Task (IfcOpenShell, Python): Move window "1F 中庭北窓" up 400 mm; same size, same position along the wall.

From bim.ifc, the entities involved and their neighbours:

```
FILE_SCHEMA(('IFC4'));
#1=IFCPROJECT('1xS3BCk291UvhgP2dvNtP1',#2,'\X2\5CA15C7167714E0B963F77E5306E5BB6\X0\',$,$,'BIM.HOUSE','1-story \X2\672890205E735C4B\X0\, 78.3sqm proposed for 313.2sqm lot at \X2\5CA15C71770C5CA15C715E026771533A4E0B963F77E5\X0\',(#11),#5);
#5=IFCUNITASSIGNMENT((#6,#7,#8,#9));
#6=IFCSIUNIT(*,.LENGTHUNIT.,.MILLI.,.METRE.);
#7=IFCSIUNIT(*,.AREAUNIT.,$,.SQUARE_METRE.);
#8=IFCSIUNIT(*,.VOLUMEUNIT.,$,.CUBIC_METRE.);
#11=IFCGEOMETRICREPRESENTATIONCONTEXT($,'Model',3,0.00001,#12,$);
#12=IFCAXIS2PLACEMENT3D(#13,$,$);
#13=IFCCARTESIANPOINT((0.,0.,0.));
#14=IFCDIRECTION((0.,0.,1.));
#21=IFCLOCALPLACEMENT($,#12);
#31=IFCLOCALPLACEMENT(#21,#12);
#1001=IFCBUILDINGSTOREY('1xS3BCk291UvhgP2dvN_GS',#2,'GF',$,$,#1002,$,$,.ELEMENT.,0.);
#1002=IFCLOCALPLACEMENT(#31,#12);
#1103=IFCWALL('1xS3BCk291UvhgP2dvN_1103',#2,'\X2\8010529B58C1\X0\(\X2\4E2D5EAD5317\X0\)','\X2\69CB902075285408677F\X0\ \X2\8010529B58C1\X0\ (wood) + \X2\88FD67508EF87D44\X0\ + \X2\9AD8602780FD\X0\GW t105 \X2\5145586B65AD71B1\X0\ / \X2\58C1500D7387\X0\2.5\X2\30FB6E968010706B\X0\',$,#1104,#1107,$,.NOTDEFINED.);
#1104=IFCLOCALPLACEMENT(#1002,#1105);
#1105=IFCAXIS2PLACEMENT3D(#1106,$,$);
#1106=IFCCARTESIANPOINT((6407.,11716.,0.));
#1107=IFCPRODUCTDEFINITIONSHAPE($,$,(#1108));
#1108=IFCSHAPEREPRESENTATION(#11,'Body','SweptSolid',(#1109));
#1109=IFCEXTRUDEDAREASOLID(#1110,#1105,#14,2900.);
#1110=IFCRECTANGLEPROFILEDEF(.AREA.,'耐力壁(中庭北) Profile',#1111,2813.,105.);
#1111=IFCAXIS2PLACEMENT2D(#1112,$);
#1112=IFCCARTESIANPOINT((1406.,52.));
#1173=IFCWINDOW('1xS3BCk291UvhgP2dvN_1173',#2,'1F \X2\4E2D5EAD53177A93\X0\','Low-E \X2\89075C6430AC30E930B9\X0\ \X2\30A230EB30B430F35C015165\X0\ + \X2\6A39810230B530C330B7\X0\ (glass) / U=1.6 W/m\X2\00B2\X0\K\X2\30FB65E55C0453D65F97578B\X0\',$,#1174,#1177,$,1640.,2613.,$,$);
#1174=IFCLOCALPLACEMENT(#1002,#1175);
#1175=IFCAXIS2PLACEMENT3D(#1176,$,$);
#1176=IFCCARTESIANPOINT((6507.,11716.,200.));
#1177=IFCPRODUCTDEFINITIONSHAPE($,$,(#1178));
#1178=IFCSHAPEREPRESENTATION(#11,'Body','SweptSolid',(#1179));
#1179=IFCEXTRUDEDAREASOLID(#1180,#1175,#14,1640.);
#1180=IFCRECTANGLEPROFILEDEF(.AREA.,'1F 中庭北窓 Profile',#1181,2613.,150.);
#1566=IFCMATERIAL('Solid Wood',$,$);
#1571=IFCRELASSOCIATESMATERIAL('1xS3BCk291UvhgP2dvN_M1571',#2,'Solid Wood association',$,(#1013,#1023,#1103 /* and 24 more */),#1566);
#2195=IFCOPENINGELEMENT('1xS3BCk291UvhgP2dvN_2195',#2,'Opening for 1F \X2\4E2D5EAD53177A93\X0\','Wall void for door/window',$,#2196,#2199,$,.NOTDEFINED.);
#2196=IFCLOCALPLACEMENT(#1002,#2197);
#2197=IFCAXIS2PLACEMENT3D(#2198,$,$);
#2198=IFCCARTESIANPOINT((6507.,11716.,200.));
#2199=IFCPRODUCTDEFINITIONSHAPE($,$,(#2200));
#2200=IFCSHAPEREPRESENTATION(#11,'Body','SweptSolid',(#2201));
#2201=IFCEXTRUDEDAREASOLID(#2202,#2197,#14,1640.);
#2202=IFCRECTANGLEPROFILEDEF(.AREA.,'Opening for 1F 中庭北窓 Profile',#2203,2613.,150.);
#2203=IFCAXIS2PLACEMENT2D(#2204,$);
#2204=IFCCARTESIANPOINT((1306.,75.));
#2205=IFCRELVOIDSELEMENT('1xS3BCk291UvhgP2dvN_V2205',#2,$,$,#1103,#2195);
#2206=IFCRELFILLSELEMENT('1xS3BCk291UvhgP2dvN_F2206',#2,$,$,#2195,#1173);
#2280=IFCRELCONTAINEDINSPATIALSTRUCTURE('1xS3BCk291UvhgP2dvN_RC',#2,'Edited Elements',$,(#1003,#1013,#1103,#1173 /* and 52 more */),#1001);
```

```python
import numpy as np
import ifcopenshell
import ifcopenshell.api.geometry
import ifcopenshell.util.placement
import ifcopenshell.util.unit

model = ifcopenshell.open("bim.ifc")
unit_scale = ifcopenshell.util.unit.calculate_unit_scale(model)

window = model.by_id(1173)
opening = window.FillsVoids[0].RelatingOpeningElement
dz = 0.4 / unit_scale

shift = np.array([0.0, 0.0, dz])
# The window is not placed relative to its opening, so move both.
for product in (opening, window):
    matrix = ifcopenshell.util.placement.get_local_placement(product.ObjectPlacement)
    matrix[:3, 3] += shift
    ifcopenshell.api.geometry.edit_object_placement(model, product=product, matrix=matrix, is_si=False)

print(f"moved by {dz * unit_scale:+.3f} m")

model.write("bim_rev.ifc")
```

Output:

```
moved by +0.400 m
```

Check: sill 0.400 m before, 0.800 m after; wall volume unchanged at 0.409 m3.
